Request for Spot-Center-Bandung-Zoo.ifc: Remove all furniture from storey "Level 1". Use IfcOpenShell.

First a look at what the model holds.

```python
import ifcopenshell
import ifcopenshell.util.element

model = ifcopenshell.open("Spot-Center-Bandung-Zoo.ifc")
print(model.schema)
storey = next(s for s in model.by_type("IfcBuildingStorey") if s.Name == "Level 1")
furniture = [e for e in ifcopenshell.util.element.get_decomposition(storey) if e.is_a("IfcFurnishingElement")]
seen = {}
for e in furniture:
    element_type = ifcopenshell.util.element.get_type(e)
    name = element_type.Name if element_type not in (None, e) else None
    seen[name] = seen.get(name, 0) + 1
for name, count in sorted(seen.items(), key=str):
    print(count, "x", name)
```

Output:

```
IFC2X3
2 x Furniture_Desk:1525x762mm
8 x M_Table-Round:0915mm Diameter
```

```python
import ifcopenshell
import ifcopenshell.api.root
import ifcopenshell.util.element

model = ifcopenshell.open("Spot-Center-Bandung-Zoo.ifc")

storey = next(s for s in model.by_type("IfcBuildingStorey") if s.Name == "Level 1")
furniture = [e for e in ifcopenshell.util.element.get_decomposition(storey) if e.is_a("IfcFurnishingElement")]

for e in furniture:
    ifcopenshell.api.root.remove_product(model, product=e)
print(len(furniture), "removed")

model.write("Spot-Center-Bandung-Zoo_updated.ifc")
```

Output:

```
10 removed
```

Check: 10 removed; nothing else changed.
